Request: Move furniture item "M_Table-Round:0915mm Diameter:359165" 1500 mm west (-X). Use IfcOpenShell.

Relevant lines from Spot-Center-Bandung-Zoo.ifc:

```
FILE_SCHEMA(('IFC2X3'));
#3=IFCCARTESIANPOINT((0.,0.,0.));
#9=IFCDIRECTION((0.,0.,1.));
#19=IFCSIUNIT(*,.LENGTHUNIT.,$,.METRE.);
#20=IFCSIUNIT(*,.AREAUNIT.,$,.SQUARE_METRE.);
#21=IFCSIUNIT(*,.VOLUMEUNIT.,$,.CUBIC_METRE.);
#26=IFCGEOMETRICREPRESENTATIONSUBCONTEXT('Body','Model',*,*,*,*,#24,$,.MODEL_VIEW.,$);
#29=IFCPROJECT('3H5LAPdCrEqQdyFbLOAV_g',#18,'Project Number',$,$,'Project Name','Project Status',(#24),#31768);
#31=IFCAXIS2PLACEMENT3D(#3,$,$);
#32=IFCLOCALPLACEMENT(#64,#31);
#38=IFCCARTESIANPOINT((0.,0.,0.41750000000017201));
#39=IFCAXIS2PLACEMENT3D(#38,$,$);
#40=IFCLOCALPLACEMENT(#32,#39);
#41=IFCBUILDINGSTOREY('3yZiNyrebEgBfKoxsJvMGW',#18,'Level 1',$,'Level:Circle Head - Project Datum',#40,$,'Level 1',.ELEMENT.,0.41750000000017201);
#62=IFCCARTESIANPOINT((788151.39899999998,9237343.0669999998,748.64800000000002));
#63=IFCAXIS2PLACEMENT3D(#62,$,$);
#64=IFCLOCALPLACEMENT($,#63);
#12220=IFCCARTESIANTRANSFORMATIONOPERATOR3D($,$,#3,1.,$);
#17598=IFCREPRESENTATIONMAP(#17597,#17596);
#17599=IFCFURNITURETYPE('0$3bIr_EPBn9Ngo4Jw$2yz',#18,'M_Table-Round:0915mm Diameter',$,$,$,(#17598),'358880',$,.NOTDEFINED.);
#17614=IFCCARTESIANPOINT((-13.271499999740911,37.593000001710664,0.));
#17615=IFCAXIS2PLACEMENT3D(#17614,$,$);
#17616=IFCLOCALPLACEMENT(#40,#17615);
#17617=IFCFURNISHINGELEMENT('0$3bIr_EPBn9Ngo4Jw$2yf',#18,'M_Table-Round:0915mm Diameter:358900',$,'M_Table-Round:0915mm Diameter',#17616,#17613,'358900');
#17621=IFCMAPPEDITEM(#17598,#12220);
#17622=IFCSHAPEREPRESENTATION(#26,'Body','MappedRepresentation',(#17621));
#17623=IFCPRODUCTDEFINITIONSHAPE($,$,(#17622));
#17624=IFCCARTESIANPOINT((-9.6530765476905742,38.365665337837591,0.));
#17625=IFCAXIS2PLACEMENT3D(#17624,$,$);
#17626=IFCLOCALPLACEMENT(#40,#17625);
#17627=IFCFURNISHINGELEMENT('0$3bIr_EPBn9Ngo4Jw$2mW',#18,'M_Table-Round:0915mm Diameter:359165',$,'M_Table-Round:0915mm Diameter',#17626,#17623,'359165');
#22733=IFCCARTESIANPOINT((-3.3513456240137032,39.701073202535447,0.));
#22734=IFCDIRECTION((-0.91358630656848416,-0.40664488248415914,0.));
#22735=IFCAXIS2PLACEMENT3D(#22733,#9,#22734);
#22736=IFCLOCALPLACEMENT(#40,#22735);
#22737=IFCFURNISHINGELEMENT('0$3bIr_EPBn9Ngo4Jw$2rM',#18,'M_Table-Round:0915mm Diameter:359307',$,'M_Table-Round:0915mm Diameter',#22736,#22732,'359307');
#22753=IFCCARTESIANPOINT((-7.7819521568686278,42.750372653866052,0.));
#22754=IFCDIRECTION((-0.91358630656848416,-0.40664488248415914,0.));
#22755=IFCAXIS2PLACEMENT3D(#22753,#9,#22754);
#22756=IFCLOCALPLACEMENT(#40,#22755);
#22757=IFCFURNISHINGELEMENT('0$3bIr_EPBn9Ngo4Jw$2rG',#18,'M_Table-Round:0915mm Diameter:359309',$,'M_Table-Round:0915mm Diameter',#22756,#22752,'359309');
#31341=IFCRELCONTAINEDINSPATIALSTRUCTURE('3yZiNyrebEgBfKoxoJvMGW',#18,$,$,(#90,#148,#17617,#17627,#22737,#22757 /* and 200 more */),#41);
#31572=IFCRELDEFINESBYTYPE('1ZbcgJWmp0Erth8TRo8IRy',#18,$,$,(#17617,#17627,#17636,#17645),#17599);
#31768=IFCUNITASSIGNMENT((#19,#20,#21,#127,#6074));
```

```python
import ifcopenshell
import ifcopenshell.api.geometry
import ifcopenshell.util.placement
import ifcopenshell.util.unit

model = ifcopenshell.open("Spot-Center-Bandung-Zoo.ifc")
unit_scale = ifcopenshell.util.unit.calculate_unit_scale(model)

item = model.by_guid("0$3bIr_EPBn9Ngo4Jw$2mW")
matrix = ifcopenshell.util.placement.get_local_placement(item.ObjectPlacement)
matrix[0, 3] -= 1.5 / unit_scale
ifcopenshell.api.geometry.edit_object_placement(model, product=item, matrix=matrix, is_si=False)

print(ifcopenshell.util.placement.get_local_placement(item.ObjectPlacement).round(3) + 0.0)

model.write("Spot-Center-Bandung-Zoo-out.ifc")
```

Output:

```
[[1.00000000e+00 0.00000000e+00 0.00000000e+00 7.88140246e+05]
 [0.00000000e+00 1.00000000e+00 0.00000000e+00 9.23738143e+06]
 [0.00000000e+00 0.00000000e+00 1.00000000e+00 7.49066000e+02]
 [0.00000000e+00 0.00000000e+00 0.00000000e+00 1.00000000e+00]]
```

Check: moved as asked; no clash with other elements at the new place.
